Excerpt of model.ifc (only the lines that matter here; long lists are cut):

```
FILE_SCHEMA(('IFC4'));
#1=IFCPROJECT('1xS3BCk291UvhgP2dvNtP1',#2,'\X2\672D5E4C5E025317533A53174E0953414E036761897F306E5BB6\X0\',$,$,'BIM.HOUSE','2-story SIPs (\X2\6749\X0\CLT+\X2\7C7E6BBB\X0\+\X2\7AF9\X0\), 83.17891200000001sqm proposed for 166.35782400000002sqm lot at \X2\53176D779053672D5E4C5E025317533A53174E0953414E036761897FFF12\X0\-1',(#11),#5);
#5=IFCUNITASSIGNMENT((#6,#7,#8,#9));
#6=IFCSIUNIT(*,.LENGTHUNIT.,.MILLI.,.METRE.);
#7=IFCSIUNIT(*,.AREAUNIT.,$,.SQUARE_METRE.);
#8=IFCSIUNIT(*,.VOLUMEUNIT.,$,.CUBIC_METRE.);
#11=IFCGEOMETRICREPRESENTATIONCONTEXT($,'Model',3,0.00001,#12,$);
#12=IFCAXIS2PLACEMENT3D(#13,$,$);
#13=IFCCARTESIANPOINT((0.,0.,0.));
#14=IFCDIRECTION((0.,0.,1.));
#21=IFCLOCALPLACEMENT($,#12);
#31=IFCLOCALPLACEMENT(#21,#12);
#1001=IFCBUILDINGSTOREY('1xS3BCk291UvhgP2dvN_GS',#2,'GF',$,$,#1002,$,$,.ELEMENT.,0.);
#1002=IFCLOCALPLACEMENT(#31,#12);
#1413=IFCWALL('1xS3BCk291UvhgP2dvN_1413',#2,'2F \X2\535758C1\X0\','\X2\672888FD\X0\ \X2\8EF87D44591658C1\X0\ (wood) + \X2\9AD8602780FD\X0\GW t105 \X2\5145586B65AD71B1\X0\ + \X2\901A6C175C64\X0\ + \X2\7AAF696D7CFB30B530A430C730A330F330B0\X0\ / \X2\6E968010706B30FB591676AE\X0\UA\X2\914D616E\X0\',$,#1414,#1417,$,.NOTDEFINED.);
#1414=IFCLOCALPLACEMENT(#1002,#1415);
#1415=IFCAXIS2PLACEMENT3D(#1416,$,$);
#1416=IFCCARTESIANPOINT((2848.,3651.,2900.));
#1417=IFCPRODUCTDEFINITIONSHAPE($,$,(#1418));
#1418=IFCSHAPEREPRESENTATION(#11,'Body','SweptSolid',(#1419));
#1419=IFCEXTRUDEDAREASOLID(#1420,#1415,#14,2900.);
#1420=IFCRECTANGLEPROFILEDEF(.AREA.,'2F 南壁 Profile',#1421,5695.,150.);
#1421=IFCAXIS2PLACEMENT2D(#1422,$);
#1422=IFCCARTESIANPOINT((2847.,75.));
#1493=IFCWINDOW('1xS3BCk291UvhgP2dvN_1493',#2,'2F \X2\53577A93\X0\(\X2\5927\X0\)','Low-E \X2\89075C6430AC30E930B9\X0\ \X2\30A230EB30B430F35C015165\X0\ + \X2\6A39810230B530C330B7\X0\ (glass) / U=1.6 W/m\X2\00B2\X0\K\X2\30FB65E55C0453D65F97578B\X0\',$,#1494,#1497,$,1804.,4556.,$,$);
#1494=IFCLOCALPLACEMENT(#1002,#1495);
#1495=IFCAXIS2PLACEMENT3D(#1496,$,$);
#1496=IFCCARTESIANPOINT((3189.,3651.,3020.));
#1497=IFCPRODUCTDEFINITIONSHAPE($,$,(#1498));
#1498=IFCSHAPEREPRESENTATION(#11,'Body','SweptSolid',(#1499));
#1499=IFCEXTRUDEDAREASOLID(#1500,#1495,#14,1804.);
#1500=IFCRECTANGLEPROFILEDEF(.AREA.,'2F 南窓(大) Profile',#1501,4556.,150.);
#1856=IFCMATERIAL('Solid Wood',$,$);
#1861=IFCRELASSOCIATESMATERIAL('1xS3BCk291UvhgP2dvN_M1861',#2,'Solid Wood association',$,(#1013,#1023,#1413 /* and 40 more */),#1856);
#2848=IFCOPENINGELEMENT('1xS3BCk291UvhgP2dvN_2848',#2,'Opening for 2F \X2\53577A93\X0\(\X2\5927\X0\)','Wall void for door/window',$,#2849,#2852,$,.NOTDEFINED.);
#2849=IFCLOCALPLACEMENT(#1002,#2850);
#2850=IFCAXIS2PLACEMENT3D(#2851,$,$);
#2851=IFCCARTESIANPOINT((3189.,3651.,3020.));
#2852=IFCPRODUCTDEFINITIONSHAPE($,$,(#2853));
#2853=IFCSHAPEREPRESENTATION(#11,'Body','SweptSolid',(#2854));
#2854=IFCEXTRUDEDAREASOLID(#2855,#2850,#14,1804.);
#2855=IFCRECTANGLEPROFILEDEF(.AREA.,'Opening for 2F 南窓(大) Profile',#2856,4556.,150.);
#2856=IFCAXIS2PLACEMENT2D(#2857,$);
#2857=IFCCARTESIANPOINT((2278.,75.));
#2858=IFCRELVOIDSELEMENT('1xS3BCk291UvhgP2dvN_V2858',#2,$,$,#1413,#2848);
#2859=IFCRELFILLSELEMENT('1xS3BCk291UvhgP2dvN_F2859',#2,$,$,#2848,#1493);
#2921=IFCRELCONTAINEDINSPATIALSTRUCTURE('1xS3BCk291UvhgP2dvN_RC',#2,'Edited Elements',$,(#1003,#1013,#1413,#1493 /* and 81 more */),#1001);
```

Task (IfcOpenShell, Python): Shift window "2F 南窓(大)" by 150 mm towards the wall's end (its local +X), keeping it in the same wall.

```python
import ifcopenshell
import ifcopenshell.api.geometry
import ifcopenshell.util.placement
import ifcopenshell.util.unit

model = ifcopenshell.open("model.ifc")
unit_scale = ifcopenshell.util.unit.calculate_unit_scale(model)

window = model.by_guid("1xS3BCk291UvhgP2dvN_1493")
opening = window.FillsVoids[0].RelatingOpeningElement
wall = opening.VoidsElements[0].RelatingBuildingElement

wall_matrix = ifcopenshell.util.placement.get_local_placement(wall.ObjectPlacement)
shift = wall_matrix[:3, 0] * 0.15 / unit_scale
before = ifcopenshell.util.placement.get_local_placement(window.ObjectPlacement)[:3, 3].copy()

# The window is not placed relative to its opening, so move both.
for product in (opening, window):
    matrix = ifcopenshell.util.placement.get_local_placement(product.ObjectPlacement)
    matrix[:3, 3] += shift
    ifcopenshell.api.geometry.edit_object_placement(model, product=product, matrix=matrix, is_si=False)

after = ifcopenshell.util.placement.get_local_placement(window.ObjectPlacement)[:3, 3]
print("window moved by", (after - before).round(3) + 0.0)

model.write("model_v2.ifc")
```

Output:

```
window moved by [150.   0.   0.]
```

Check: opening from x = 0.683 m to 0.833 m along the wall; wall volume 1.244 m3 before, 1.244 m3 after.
